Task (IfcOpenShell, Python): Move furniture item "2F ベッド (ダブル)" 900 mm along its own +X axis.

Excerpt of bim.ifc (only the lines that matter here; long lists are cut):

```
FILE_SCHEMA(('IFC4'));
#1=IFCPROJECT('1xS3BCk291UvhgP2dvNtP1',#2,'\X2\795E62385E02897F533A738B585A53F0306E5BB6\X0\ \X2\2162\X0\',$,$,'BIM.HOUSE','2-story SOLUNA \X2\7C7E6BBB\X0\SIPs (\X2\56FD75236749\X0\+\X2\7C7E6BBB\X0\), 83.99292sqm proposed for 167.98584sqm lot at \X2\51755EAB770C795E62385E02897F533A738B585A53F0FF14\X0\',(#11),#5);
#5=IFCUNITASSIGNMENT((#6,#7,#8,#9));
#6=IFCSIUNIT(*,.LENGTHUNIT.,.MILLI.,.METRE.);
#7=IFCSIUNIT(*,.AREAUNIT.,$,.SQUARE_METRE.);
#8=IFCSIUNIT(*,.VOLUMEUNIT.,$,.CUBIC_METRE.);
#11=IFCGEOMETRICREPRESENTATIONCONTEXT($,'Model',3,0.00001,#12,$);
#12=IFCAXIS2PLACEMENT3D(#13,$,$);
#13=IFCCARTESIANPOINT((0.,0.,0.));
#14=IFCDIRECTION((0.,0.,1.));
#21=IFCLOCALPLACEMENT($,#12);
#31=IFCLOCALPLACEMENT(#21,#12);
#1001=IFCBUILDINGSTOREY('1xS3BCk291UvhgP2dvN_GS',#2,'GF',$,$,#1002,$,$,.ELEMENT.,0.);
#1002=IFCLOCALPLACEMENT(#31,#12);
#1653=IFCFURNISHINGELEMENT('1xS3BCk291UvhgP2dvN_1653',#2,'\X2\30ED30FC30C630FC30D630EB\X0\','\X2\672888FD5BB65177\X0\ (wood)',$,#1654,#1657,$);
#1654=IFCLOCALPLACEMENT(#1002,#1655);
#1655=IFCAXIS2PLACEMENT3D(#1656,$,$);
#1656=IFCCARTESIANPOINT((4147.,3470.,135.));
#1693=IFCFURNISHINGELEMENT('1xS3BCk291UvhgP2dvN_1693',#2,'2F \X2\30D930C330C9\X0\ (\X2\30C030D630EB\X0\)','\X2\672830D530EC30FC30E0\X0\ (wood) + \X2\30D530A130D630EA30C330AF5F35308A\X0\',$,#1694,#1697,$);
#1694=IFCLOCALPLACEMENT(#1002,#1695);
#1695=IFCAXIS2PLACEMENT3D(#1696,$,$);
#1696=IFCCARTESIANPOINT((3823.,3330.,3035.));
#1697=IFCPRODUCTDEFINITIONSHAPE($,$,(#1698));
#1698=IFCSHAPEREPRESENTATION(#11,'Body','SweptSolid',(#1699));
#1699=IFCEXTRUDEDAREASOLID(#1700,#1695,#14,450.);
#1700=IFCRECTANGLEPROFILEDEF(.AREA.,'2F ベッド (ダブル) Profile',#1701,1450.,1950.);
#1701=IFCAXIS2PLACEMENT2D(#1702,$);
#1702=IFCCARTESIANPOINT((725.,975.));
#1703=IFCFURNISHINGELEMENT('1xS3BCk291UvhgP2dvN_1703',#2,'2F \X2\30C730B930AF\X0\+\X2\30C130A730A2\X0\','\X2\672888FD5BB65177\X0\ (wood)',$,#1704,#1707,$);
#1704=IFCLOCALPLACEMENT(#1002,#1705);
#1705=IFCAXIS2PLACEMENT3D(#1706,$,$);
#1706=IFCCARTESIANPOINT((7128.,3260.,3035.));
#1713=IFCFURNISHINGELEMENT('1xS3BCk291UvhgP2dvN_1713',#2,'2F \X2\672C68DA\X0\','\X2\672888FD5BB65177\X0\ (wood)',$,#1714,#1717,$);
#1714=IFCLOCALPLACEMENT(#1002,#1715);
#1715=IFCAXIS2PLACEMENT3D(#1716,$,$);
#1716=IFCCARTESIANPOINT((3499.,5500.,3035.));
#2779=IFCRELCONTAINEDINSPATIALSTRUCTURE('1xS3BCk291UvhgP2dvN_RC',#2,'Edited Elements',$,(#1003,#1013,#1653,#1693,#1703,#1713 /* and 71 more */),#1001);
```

```python
import ifcopenshell
import ifcopenshell.api.geometry
import ifcopenshell.util.placement

model = ifcopenshell.open("bim.ifc")

item = model.by_guid("1xS3BCk291UvhgP2dvN_1693")
matrix = ifcopenshell.util.placement.get_local_placement(item.ObjectPlacement)
matrix[:3, 3] += matrix[:3, 0] * 900.0
ifcopenshell.api.geometry.edit_object_placement(model, product=item, matrix=matrix, is_si=False)

print(ifcopenshell.util.placement.get_local_placement(item.ObjectPlacement).round(3) + 0.0)

model.write("bim_rev.ifc")
```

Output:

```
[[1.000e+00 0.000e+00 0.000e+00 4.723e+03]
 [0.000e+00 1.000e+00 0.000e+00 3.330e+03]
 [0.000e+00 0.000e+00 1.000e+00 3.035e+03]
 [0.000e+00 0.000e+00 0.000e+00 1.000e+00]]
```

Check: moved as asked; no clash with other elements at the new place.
